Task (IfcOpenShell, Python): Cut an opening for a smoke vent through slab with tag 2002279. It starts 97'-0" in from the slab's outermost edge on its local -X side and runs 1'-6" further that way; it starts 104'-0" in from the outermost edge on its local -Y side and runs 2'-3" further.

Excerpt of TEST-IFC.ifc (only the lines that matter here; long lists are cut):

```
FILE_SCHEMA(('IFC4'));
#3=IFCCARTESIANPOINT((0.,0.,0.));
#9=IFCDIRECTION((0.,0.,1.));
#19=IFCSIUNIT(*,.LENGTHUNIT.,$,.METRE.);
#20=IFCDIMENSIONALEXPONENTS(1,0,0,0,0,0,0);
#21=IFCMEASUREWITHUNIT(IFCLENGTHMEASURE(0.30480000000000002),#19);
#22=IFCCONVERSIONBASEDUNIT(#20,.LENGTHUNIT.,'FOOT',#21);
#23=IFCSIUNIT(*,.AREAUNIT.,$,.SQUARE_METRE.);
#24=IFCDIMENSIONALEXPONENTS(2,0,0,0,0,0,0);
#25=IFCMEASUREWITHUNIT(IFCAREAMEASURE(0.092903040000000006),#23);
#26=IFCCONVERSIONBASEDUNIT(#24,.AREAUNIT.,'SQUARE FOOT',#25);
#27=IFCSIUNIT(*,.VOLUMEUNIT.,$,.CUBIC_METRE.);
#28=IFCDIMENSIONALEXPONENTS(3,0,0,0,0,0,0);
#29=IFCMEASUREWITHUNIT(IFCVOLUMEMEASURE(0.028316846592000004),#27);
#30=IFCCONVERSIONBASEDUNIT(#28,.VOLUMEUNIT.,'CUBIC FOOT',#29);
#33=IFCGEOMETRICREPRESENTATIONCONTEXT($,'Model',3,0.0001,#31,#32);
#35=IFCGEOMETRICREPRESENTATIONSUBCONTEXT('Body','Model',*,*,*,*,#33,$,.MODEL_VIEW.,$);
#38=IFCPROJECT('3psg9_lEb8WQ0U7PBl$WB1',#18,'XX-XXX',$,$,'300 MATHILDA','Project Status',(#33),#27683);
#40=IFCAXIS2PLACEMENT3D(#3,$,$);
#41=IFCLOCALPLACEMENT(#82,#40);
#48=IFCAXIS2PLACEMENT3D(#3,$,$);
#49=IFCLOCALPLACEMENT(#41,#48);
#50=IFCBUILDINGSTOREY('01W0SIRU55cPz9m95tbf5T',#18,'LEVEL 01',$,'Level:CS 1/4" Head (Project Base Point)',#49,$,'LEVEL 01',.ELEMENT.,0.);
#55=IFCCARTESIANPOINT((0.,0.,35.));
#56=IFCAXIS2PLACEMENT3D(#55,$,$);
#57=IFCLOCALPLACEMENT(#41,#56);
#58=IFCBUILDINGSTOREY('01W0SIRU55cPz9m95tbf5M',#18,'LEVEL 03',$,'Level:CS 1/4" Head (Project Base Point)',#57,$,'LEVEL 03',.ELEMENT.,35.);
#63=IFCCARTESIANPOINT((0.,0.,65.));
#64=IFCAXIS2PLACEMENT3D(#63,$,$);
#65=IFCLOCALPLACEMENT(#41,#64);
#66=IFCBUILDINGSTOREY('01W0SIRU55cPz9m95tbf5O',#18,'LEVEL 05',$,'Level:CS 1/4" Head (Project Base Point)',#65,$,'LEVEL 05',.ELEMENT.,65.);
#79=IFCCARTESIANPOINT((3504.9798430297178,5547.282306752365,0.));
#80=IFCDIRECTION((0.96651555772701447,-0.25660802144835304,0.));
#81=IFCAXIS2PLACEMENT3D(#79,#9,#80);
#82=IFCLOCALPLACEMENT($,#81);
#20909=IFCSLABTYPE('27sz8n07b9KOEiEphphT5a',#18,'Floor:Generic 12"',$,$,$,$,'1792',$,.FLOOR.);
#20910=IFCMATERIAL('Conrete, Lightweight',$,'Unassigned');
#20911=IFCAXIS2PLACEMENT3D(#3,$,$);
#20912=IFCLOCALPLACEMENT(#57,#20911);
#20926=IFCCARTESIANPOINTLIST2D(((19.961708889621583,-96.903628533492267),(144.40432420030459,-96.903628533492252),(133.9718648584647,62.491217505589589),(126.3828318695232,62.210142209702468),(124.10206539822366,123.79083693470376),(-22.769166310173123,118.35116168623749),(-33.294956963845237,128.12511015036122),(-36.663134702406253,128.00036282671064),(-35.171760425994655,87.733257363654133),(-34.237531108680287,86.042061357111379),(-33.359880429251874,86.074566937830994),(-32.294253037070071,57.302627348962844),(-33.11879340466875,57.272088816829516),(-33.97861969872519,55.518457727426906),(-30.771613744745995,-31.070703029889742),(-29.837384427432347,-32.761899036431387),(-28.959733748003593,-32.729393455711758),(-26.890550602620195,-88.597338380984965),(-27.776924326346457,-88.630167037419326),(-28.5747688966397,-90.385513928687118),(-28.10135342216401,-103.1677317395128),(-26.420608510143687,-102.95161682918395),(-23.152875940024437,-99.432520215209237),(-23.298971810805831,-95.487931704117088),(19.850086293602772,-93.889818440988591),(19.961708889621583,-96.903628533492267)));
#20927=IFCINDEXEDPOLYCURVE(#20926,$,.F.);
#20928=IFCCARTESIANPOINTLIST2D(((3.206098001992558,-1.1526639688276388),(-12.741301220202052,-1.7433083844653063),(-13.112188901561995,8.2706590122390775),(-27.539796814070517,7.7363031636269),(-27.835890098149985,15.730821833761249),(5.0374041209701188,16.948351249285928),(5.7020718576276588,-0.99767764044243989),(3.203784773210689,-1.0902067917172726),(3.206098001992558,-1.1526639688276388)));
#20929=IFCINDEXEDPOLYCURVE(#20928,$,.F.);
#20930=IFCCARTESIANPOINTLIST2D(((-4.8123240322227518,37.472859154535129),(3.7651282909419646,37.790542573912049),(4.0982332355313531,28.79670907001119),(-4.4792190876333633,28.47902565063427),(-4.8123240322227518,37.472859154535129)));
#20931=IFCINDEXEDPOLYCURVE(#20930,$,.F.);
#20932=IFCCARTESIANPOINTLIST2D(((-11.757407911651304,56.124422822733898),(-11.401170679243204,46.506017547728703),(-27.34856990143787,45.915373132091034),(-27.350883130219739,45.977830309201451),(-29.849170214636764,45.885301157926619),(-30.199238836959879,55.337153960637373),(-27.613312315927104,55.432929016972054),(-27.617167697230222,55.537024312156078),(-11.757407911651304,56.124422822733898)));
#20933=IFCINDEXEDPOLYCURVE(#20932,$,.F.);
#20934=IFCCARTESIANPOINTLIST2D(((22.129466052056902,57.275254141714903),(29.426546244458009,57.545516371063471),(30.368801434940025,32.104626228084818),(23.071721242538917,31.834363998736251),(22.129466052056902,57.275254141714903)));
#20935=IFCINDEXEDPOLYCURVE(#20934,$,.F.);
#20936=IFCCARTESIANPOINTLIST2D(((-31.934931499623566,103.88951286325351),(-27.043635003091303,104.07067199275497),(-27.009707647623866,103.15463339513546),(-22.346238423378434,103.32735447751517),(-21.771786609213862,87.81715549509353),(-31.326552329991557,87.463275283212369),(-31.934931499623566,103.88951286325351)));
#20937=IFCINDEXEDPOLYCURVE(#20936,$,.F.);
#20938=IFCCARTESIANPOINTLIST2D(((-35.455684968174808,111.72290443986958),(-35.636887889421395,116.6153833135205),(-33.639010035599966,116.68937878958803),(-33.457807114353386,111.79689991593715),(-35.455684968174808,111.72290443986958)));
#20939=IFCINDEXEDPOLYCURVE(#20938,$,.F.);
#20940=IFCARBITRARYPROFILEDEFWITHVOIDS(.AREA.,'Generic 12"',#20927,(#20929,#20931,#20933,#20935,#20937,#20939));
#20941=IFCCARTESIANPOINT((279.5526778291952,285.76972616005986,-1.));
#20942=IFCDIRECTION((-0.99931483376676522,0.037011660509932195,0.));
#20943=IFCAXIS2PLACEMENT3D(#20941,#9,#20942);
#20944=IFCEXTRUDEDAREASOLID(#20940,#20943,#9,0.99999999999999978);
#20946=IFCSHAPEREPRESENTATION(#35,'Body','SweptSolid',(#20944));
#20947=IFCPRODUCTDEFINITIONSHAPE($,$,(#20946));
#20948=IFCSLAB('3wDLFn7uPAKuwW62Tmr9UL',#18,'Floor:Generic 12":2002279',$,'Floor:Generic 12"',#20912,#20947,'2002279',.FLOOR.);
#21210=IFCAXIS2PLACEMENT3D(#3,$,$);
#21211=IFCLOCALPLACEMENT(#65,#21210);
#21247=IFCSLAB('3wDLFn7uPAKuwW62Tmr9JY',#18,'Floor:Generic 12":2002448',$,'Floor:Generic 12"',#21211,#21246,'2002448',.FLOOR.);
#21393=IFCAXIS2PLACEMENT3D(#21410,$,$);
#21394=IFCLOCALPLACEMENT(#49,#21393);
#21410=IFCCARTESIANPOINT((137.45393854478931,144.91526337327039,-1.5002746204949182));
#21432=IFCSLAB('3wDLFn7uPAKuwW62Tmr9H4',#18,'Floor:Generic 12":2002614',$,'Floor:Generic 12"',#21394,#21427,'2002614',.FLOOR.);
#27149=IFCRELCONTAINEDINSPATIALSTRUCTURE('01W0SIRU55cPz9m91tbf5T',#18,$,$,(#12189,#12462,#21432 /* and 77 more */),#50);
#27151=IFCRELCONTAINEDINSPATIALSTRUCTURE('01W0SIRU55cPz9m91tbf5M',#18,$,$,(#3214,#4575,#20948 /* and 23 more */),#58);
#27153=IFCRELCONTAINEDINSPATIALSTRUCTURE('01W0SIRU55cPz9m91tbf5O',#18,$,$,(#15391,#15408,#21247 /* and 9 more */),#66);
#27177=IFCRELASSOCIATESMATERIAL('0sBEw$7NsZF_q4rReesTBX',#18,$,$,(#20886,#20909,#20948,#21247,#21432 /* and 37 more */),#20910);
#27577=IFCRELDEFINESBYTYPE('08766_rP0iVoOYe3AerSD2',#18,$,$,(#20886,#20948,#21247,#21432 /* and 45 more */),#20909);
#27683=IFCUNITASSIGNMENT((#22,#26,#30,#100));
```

```python
import numpy as np
import ifcopenshell
import ifcopenshell.api.feature
import ifcopenshell.api.geometry
import ifcopenshell.api.root
import ifcopenshell.geom
import ifcopenshell.util.placement
import ifcopenshell.util.representation
import ifcopenshell.util.shape
import ifcopenshell.util.unit

model = ifcopenshell.open("TEST-IFC.ifc")
unit_scale = ifcopenshell.util.unit.calculate_unit_scale(model)
settings = ifcopenshell.geom.settings()


def volume(element):
    """Net volume in cubic metres, openings subtracted."""
    shape = ifcopenshell.geom.create_shape(settings, element)
    return ifcopenshell.util.shape.get_volume(shape.geometry)


slab = model.by_guid("3wDLFn7uPAKuwW62Tmr9UL")
before = volume(slab)

# Extent in the slab's own axes, in metres. The edges named are its -X and -Y sides.
slab_shape = ifcopenshell.geom.create_shape(settings, slab)
vertices = ifcopenshell.util.shape.get_vertices(slab_shape.geometry)
x_min, y_min, bottom = vertices.min(axis=0)
top = vertices[:, 2].max()

opening = ifcopenshell.api.root.create_entity(model, ifc_class="IfcOpeningElement", name="Smoke vent opening", predefined_type="OPENING")
context = ifcopenshell.util.representation.get_context(model, "Model", "Body", "MODEL_VIEW")
width, depth = 0.4572, 0.6858
outline = [(0.0, 0.0), (width, 0.0), (width, depth), (0.0, depth), (0.0, 0.0)]
# Overshoot both faces by 50 mm so the cut is clean.
shape = ifcopenshell.api.geometry.add_slab_representation(
    model, context=context, depth=top - bottom + 0.1, polyline=outline
)
ifcopenshell.api.geometry.assign_representation(model, product=opening, representation=shape)

matrix = ifcopenshell.util.placement.get_local_placement(slab.ObjectPlacement)
matrix[:, 3] = matrix @ np.append(np.array([x_min + 29.5656, y_min + 31.6992, bottom - 0.05]) / unit_scale, 1.0)
ifcopenshell.api.geometry.edit_object_placement(model, product=opening, matrix=matrix, is_si=False)
ifcopenshell.api.feature.add_feature(model, feature=opening, element=slab)

after = volume(slab)

print(f"slab volume {before:.3f} -> {after:.3f} m3")

model.write("TEST-IFC_rev.ifc")
```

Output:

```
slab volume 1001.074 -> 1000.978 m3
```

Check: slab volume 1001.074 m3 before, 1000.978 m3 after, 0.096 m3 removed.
